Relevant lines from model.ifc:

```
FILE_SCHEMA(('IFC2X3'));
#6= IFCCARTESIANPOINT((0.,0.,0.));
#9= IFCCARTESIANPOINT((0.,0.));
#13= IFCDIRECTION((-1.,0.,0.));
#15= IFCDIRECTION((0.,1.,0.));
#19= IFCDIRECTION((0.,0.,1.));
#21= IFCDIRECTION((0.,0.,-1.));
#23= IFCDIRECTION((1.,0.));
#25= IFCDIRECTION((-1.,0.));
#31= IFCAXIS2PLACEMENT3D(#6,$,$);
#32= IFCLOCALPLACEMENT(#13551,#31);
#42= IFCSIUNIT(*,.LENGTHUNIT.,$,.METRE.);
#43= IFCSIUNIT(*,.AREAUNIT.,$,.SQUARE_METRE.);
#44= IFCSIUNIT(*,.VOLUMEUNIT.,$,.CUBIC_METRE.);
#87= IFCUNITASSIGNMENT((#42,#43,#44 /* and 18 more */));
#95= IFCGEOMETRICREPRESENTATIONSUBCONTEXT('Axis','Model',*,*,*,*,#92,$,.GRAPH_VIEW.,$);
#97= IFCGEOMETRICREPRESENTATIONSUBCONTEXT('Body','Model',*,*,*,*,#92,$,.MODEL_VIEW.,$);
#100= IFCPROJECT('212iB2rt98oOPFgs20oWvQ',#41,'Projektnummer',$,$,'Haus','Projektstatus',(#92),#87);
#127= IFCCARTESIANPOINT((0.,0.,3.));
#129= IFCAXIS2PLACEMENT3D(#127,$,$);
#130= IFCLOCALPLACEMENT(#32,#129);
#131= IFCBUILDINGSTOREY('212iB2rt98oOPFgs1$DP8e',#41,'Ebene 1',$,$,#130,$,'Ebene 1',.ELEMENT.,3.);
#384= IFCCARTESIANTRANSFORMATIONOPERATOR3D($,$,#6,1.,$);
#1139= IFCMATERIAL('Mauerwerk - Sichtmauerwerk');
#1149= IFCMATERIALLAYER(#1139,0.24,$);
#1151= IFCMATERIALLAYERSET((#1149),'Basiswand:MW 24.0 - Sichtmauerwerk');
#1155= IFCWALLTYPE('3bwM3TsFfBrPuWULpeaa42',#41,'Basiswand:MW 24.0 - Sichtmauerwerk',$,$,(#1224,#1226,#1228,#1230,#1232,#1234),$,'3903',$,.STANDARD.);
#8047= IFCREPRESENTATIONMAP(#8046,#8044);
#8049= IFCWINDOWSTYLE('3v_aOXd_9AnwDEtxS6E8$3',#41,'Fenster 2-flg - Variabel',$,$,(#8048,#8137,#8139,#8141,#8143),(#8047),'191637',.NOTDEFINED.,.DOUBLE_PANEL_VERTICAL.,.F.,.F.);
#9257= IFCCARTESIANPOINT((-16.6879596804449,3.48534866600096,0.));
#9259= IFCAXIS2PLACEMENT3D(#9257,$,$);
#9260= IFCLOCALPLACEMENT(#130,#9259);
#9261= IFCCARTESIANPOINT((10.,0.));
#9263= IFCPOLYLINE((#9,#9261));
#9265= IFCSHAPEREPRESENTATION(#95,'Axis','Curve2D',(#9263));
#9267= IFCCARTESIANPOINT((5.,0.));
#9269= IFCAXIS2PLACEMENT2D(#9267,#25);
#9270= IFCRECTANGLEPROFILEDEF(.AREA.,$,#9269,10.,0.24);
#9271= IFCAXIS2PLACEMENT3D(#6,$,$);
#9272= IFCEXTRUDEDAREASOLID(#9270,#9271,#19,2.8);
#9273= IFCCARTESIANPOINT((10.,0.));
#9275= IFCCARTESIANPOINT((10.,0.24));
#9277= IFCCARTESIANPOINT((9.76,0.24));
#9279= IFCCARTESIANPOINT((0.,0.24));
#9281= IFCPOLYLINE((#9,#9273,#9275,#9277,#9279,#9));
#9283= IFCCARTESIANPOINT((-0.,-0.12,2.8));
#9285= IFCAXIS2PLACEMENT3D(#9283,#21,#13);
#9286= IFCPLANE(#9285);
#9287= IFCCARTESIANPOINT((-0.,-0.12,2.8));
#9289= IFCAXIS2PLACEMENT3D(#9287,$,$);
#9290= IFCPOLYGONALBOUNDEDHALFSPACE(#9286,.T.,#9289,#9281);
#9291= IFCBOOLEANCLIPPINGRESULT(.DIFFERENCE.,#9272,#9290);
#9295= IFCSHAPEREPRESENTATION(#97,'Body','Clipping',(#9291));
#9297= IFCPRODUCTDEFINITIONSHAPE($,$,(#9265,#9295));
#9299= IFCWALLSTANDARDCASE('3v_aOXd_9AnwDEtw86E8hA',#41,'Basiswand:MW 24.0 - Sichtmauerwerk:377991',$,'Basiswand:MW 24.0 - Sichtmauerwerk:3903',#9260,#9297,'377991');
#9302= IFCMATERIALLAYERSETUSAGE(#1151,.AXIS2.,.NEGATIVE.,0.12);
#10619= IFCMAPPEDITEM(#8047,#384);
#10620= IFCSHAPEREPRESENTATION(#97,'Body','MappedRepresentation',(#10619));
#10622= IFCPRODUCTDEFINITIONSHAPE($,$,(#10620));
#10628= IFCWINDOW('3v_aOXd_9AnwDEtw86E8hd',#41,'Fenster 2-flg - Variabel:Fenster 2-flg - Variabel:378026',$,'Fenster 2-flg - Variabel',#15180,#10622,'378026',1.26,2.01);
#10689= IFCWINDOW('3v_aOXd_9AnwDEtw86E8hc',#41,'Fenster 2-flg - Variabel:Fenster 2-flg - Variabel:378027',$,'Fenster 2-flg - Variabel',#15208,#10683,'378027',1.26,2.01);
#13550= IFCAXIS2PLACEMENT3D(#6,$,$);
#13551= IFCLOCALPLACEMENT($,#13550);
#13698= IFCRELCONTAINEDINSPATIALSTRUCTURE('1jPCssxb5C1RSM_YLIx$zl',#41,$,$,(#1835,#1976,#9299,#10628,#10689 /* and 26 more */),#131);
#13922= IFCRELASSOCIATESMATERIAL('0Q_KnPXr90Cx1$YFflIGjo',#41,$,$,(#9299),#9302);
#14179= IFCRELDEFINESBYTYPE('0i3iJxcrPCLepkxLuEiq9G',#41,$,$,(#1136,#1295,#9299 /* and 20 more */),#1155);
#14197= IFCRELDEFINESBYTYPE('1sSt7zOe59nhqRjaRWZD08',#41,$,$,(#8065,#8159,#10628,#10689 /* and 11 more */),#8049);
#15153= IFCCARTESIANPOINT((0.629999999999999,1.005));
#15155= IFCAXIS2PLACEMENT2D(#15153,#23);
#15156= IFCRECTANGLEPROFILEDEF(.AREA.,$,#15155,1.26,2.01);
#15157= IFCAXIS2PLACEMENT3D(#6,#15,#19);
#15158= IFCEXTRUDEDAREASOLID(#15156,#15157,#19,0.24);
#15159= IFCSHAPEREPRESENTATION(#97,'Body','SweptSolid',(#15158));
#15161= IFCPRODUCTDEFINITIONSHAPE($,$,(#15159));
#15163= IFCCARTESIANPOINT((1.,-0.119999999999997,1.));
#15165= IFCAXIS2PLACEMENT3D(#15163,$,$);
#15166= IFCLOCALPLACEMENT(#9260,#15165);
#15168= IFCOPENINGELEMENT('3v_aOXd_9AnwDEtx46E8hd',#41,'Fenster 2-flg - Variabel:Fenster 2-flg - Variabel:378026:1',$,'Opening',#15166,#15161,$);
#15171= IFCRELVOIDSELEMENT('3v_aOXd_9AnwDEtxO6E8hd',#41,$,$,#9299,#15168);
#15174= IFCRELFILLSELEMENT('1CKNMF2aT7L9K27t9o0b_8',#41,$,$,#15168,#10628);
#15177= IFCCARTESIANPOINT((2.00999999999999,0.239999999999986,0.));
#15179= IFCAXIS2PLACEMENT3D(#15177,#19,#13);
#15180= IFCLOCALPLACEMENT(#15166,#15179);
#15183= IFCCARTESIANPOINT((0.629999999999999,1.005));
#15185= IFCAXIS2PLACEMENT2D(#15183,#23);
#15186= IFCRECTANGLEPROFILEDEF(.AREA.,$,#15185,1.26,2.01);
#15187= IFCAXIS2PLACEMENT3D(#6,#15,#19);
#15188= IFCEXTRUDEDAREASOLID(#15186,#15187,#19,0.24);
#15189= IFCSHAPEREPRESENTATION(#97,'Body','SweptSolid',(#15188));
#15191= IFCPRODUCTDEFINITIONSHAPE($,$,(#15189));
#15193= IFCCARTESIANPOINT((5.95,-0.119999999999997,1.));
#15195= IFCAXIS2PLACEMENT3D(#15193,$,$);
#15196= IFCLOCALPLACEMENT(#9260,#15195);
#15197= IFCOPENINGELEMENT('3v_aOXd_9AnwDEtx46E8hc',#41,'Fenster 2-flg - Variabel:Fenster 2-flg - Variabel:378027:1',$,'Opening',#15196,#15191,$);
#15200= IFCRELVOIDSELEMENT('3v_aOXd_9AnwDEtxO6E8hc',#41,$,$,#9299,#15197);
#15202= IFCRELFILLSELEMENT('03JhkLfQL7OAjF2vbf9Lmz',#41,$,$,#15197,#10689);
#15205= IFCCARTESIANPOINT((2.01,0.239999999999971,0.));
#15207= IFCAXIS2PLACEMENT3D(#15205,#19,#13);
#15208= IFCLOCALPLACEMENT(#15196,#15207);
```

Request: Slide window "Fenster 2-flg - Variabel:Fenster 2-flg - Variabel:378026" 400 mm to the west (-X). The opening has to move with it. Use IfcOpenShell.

```python
import ifcopenshell
import ifcopenshell.api.geometry
import ifcopenshell.util.placement

model = ifcopenshell.open("model.ifc")

window = model.by_guid("3v_aOXd_9AnwDEtw86E8hd")
opening = window.FillsVoids[0].RelatingOpeningElement
wall = opening.VoidsElements[0].RelatingBuildingElement

wall_matrix = ifcopenshell.util.placement.get_local_placement(wall.ObjectPlacement)
shift = wall_matrix[:3, 0] * -0.4
before = ifcopenshell.util.placement.get_local_placement(window.ObjectPlacement)[:3, 3].copy()

# The window is placed relative to its opening, so it follows when the opening moves.
matrix = ifcopenshell.util.placement.get_local_placement(opening.ObjectPlacement)
matrix[:3, 3] += shift
ifcopenshell.api.geometry.edit_object_placement(
    model, product=opening, matrix=matrix, is_si=False, should_transform_children=True
)

after = ifcopenshell.util.placement.get_local_placement(window.ObjectPlacement)[:3, 3]
print("window moved by", (after - before).round(3) + 0.0)

model.write("model_updated.ifc")
```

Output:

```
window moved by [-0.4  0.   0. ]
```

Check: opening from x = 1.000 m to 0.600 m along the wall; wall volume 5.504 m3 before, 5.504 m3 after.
